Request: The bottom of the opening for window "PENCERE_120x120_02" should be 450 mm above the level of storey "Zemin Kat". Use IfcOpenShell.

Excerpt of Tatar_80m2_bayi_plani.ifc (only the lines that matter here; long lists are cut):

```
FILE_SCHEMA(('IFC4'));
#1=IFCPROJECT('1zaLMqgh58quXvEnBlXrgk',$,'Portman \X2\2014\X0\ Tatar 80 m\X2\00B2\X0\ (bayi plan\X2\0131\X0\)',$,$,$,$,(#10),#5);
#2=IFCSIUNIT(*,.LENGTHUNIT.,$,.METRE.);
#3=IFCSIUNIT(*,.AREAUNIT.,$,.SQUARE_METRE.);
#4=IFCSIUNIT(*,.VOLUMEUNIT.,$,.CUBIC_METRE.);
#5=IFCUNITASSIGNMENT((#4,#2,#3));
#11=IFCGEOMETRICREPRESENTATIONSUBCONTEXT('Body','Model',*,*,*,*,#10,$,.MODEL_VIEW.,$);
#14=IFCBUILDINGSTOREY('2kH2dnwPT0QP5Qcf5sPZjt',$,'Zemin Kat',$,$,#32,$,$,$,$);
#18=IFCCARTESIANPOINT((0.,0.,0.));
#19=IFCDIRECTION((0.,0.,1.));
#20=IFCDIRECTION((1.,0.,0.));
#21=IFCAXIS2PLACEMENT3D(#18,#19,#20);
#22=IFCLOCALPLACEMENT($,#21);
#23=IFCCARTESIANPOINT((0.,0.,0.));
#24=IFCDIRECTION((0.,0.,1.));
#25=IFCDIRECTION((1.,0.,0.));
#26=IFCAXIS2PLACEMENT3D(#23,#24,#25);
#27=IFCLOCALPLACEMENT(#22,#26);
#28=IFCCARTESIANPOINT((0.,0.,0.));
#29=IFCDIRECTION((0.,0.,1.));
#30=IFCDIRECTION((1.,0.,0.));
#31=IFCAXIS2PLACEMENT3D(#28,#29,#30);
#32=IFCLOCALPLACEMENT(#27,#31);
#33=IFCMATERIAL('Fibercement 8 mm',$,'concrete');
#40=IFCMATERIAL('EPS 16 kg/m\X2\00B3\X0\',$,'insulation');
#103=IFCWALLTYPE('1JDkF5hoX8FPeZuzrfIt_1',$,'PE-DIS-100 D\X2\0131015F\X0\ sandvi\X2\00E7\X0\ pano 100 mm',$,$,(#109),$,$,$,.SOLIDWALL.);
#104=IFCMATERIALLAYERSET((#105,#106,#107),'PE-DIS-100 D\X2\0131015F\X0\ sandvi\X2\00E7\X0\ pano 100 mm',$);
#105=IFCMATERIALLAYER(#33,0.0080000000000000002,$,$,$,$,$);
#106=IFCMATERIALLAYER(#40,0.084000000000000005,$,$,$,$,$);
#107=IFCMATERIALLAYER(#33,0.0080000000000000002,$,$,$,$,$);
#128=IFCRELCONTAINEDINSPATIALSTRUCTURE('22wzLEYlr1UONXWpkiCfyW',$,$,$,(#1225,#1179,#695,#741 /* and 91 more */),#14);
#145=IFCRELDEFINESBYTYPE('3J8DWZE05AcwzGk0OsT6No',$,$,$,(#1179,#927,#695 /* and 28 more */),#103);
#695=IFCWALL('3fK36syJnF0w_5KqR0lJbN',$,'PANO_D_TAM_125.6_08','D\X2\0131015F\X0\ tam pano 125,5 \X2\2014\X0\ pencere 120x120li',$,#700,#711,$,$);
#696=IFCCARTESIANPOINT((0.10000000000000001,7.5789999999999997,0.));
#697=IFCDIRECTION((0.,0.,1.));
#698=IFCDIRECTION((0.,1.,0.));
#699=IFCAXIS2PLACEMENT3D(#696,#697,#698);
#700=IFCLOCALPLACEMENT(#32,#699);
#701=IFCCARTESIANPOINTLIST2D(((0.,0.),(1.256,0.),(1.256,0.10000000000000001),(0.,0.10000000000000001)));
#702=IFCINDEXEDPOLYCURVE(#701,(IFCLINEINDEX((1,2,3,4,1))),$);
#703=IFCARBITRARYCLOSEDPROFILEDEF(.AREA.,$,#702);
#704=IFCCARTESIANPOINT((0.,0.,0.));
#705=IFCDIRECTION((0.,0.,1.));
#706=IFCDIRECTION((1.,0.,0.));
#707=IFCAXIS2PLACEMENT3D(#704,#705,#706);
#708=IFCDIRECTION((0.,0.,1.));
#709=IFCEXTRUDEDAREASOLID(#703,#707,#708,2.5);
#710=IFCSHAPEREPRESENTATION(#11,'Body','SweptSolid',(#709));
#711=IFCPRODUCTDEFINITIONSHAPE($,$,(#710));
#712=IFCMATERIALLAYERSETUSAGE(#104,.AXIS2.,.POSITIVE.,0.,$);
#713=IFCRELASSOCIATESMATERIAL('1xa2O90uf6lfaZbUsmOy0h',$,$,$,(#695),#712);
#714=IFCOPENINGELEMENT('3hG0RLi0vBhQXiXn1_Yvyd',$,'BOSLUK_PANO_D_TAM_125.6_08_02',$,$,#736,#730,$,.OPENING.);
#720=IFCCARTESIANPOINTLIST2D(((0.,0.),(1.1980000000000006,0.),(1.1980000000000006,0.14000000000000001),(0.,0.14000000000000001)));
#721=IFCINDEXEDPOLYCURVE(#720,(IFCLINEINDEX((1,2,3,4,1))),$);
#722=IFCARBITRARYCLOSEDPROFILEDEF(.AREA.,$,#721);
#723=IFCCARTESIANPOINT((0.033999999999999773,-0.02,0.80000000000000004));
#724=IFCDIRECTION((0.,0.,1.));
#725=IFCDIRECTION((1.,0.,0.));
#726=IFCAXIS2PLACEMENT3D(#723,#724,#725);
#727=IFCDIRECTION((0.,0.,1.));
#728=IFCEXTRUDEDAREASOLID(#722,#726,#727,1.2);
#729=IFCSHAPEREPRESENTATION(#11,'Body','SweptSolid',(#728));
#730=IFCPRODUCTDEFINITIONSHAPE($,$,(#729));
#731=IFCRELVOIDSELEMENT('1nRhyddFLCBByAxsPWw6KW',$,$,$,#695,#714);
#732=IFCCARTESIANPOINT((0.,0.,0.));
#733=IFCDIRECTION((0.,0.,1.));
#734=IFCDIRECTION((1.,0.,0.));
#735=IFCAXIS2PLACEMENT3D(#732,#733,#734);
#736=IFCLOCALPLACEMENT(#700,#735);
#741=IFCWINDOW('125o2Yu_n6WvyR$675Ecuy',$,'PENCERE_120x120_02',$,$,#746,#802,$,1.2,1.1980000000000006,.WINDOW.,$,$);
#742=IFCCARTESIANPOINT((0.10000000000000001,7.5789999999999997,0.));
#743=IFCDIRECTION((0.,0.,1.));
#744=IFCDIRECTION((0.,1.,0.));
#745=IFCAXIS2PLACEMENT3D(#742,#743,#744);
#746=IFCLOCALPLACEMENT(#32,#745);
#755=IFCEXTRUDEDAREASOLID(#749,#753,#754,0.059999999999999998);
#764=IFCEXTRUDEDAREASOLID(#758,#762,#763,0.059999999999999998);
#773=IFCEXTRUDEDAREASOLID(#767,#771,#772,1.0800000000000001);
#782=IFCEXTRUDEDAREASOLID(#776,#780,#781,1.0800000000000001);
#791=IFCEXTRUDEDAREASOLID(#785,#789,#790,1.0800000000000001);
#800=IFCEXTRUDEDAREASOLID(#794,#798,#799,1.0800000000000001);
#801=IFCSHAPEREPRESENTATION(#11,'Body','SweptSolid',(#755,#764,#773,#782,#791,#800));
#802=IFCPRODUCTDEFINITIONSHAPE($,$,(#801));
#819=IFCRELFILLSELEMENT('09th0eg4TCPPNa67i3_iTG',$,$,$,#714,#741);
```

```python
import numpy as np
import ifcopenshell
import ifcopenshell.api.geometry
import ifcopenshell.geom
import ifcopenshell.util.element
import ifcopenshell.util.placement
import ifcopenshell.util.shape
import ifcopenshell.util.unit

model = ifcopenshell.open("Tatar_80m2_bayi_plani.ifc")
unit_scale = ifcopenshell.util.unit.calculate_unit_scale(model)

window = model.by_guid("125o2Yu_n6WvyR$675Ecuy")
opening = window.FillsVoids[0].RelatingOpeningElement
storey = ifcopenshell.util.element.get_container(window, ifc_class="IfcBuildingStorey")
level = ifcopenshell.util.placement.get_local_placement(storey.ObjectPlacement)[2, 3]

# The opening's origin need not be at the sill, so measure its lowest point.
shape = ifcopenshell.geom.create_shape(ifcopenshell.geom.settings(), opening)
bottom = ifcopenshell.util.shape.get_shape_bottom_elevation(shape, shape.geometry) / unit_scale
dz = level + 0.45 / unit_scale - bottom

shift = np.array([0.0, 0.0, dz])
# The window is not placed relative to its opening, so move both.
for product in (opening, window):
    matrix = ifcopenshell.util.placement.get_local_placement(product.ObjectPlacement)
    matrix[:3, 3] += shift
    ifcopenshell.api.geometry.edit_object_placement(model, product=product, matrix=matrix, is_si=False)

print(f"moved by {dz * unit_scale:+.3f} m")

model.write("Tatar_80m2_bayi_plani_updated.ifc")
```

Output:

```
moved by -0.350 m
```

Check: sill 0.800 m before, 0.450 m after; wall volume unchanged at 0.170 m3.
